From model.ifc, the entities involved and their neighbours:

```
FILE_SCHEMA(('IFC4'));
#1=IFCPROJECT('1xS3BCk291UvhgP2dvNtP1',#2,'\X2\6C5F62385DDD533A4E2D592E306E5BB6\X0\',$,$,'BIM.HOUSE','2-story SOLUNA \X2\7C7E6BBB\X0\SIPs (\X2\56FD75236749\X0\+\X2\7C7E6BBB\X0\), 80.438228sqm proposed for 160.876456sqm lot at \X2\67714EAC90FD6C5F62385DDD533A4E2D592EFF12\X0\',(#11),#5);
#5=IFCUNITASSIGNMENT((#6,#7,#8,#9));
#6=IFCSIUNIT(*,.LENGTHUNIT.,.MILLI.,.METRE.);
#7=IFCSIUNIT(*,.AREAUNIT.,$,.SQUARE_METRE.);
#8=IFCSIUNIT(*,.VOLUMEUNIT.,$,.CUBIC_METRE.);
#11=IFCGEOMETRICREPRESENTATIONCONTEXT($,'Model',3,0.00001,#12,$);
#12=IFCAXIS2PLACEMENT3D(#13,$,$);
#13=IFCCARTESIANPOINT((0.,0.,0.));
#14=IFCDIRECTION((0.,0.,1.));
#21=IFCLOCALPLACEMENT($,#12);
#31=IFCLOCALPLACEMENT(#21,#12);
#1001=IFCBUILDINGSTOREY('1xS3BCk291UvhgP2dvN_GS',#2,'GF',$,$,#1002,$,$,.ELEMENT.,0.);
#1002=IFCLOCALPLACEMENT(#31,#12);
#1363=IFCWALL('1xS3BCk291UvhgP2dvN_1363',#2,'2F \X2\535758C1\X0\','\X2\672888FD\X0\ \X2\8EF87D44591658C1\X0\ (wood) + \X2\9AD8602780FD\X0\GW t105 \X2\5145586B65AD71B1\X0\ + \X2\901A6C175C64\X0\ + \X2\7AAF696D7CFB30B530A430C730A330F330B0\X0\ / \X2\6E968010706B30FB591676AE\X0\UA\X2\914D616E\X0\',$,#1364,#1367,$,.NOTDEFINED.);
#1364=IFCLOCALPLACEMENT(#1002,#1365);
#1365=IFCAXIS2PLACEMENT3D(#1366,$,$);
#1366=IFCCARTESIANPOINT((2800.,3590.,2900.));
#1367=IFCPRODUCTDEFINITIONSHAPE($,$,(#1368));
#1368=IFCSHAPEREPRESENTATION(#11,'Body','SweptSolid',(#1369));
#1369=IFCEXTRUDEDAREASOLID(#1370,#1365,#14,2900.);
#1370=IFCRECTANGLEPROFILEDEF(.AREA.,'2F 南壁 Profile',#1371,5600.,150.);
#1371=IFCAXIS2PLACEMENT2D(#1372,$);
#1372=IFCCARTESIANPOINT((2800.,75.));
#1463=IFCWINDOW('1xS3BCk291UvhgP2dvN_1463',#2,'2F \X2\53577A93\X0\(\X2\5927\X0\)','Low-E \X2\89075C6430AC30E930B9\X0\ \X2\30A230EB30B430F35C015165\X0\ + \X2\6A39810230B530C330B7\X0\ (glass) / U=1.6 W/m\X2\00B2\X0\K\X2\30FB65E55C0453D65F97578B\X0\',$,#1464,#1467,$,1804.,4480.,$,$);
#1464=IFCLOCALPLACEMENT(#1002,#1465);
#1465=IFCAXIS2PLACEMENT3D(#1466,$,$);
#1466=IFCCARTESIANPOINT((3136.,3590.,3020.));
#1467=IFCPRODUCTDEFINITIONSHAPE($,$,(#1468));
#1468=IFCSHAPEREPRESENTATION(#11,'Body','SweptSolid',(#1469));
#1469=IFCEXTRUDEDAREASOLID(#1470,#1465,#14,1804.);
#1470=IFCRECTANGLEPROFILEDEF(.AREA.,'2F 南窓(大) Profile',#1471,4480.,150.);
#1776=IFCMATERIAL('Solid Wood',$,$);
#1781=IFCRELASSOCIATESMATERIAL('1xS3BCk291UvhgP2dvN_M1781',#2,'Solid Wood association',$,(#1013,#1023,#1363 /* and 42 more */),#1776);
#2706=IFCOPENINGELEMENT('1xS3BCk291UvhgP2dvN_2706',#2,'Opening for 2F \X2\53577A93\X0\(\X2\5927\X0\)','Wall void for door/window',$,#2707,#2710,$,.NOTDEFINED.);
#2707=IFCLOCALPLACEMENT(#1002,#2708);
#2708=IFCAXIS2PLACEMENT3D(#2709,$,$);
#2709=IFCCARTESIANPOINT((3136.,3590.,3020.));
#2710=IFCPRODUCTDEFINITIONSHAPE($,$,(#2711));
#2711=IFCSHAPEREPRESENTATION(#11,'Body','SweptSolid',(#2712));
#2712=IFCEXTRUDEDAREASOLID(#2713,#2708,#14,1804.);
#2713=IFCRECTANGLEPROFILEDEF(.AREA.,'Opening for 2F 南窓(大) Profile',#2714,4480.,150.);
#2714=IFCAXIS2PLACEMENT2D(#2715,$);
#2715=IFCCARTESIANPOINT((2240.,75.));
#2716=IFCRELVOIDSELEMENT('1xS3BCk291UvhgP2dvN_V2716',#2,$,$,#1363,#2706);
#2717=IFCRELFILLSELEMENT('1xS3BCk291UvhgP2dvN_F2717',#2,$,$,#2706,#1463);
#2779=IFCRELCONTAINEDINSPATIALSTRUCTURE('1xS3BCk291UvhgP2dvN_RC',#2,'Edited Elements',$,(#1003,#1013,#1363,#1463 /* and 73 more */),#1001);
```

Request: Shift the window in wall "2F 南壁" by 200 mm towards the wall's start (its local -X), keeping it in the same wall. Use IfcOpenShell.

```python
import ifcopenshell
import ifcopenshell.api.geometry
import ifcopenshell.util.placement
import ifcopenshell.util.unit

model = ifcopenshell.open("model.ifc")
unit_scale = ifcopenshell.util.unit.calculate_unit_scale(model)

window = model.by_guid("1xS3BCk291UvhgP2dvN_1463")
opening = window.FillsVoids[0].RelatingOpeningElement
wall = opening.VoidsElements[0].RelatingBuildingElement

wall_matrix = ifcopenshell.util.placement.get_local_placement(wall.ObjectPlacement)
shift = wall_matrix[:3, 0] * -0.2 / unit_scale
before = ifcopenshell.util.placement.get_local_placement(window.ObjectPlacement)[:3, 3].copy()

# The window is not placed relative to its opening, so move both.
for product in (opening, window):
    matrix = ifcopenshell.util.placement.get_local_placement(product.ObjectPlacement)
    matrix[:3, 3] += shift
    ifcopenshell.api.geometry.edit_object_placement(model, product=product, matrix=matrix, is_si=False)

after = ifcopenshell.util.placement.get_local_placement(window.ObjectPlacement)[:3, 3]
print("window moved by", (after - before).round(3) + 0.0)

model.write("model_v2.ifc")
```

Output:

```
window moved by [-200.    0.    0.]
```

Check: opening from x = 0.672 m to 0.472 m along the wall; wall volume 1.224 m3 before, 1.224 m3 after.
